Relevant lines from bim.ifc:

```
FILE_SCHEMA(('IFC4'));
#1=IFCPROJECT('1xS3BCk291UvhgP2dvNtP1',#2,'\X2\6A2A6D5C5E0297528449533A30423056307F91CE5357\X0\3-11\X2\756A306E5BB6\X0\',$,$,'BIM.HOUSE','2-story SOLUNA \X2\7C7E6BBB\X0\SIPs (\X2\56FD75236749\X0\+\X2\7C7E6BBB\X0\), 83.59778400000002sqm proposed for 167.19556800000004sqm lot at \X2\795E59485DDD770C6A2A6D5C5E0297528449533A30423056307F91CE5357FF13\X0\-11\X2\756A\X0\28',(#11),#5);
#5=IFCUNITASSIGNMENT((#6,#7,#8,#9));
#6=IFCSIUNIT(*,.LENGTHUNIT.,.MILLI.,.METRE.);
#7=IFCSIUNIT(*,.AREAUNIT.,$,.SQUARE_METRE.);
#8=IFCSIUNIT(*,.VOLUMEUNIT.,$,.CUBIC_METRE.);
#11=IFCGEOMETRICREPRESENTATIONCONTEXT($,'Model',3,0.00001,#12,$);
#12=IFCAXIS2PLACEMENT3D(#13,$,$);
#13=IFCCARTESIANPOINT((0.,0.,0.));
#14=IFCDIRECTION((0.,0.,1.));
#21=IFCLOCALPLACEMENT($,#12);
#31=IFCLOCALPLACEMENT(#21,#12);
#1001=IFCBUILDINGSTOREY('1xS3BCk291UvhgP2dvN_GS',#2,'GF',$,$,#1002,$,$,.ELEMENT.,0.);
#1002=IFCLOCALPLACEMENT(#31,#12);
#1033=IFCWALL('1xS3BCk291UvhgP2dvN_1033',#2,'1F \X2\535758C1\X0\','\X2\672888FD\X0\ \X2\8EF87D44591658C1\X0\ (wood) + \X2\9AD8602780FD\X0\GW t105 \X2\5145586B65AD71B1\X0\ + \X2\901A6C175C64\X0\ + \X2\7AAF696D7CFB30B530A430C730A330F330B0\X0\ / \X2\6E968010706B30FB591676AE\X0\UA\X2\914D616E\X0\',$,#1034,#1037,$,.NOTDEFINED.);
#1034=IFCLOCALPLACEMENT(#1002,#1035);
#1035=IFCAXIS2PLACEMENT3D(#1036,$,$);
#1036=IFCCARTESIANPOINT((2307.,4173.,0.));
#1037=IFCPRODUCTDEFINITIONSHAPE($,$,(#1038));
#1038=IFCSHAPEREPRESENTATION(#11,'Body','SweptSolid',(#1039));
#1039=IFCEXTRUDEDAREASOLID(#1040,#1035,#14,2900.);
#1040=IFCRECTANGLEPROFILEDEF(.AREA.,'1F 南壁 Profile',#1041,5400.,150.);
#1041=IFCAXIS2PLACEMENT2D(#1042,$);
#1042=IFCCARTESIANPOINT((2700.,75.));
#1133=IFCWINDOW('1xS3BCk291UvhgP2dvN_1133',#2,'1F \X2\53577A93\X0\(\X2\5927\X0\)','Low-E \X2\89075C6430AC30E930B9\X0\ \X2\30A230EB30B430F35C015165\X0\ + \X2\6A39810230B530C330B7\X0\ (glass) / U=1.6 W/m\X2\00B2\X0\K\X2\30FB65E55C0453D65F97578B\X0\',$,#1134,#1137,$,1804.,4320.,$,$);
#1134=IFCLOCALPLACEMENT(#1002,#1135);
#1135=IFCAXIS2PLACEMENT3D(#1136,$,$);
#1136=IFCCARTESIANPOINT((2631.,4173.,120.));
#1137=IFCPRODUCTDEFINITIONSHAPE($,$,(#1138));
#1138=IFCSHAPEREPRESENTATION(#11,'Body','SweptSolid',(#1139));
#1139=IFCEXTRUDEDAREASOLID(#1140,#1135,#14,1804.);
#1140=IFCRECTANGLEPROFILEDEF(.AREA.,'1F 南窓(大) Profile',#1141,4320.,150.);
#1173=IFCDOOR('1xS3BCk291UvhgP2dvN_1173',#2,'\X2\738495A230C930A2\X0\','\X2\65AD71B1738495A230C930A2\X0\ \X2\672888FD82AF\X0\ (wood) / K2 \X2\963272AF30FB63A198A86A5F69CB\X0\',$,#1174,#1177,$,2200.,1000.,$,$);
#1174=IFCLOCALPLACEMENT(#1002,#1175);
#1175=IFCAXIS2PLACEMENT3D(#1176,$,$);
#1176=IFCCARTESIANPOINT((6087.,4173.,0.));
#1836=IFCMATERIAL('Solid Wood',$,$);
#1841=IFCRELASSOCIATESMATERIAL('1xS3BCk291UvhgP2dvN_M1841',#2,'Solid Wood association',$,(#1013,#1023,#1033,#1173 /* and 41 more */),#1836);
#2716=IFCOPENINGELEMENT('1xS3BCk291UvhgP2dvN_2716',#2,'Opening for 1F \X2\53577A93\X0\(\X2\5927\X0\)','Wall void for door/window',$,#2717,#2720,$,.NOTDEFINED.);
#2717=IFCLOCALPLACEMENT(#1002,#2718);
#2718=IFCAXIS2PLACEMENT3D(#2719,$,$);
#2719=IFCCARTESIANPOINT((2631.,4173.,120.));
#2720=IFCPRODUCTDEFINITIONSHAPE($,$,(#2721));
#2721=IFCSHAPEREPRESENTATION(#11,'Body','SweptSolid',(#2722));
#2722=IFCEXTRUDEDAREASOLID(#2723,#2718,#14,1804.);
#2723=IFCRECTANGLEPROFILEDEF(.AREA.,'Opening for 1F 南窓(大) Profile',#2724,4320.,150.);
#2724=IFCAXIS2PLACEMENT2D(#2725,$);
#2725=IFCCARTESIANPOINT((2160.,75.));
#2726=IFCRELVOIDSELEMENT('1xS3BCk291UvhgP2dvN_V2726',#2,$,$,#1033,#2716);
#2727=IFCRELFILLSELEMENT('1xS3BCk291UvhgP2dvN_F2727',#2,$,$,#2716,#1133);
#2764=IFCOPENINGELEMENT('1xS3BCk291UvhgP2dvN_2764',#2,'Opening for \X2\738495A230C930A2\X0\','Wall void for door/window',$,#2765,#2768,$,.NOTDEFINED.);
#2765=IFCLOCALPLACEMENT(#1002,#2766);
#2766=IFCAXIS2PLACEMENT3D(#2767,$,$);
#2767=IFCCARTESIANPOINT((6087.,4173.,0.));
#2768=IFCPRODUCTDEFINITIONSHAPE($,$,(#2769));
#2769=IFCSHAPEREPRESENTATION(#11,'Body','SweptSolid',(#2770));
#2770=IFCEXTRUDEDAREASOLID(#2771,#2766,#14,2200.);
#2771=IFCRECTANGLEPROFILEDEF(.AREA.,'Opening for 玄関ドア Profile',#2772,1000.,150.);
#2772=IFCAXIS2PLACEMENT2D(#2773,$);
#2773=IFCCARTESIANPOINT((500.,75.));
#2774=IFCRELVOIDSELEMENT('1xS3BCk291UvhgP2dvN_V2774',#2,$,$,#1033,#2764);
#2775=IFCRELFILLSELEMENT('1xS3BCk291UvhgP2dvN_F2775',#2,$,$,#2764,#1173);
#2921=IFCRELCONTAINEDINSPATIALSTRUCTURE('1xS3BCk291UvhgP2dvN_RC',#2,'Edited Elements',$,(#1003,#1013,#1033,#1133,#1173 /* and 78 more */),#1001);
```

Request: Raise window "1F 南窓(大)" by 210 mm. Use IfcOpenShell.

```python
import numpy as np
import ifcopenshell
import ifcopenshell.api.geometry
import ifcopenshell.util.placement
import ifcopenshell.util.unit

model = ifcopenshell.open("bim.ifc")
unit_scale = ifcopenshell.util.unit.calculate_unit_scale(model)

window = model.by_guid("1xS3BCk291UvhgP2dvN_1133")
opening = window.FillsVoids[0].RelatingOpeningElement
dz = 210.0

shift = np.array([0.0, 0.0, dz])
# The window is not placed relative to its opening, so move both.
for product in (opening, window):
    matrix = ifcopenshell.util.placement.get_local_placement(product.ObjectPlacement)
    matrix[:3, 3] += shift
    ifcopenshell.api.geometry.edit_object_placement(model, product=product, matrix=matrix, is_si=False)

print(f"moved by {dz * unit_scale:+.3f} m")

model.write("bim_v2.ifc")
```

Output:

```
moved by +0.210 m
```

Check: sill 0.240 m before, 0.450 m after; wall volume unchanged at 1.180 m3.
